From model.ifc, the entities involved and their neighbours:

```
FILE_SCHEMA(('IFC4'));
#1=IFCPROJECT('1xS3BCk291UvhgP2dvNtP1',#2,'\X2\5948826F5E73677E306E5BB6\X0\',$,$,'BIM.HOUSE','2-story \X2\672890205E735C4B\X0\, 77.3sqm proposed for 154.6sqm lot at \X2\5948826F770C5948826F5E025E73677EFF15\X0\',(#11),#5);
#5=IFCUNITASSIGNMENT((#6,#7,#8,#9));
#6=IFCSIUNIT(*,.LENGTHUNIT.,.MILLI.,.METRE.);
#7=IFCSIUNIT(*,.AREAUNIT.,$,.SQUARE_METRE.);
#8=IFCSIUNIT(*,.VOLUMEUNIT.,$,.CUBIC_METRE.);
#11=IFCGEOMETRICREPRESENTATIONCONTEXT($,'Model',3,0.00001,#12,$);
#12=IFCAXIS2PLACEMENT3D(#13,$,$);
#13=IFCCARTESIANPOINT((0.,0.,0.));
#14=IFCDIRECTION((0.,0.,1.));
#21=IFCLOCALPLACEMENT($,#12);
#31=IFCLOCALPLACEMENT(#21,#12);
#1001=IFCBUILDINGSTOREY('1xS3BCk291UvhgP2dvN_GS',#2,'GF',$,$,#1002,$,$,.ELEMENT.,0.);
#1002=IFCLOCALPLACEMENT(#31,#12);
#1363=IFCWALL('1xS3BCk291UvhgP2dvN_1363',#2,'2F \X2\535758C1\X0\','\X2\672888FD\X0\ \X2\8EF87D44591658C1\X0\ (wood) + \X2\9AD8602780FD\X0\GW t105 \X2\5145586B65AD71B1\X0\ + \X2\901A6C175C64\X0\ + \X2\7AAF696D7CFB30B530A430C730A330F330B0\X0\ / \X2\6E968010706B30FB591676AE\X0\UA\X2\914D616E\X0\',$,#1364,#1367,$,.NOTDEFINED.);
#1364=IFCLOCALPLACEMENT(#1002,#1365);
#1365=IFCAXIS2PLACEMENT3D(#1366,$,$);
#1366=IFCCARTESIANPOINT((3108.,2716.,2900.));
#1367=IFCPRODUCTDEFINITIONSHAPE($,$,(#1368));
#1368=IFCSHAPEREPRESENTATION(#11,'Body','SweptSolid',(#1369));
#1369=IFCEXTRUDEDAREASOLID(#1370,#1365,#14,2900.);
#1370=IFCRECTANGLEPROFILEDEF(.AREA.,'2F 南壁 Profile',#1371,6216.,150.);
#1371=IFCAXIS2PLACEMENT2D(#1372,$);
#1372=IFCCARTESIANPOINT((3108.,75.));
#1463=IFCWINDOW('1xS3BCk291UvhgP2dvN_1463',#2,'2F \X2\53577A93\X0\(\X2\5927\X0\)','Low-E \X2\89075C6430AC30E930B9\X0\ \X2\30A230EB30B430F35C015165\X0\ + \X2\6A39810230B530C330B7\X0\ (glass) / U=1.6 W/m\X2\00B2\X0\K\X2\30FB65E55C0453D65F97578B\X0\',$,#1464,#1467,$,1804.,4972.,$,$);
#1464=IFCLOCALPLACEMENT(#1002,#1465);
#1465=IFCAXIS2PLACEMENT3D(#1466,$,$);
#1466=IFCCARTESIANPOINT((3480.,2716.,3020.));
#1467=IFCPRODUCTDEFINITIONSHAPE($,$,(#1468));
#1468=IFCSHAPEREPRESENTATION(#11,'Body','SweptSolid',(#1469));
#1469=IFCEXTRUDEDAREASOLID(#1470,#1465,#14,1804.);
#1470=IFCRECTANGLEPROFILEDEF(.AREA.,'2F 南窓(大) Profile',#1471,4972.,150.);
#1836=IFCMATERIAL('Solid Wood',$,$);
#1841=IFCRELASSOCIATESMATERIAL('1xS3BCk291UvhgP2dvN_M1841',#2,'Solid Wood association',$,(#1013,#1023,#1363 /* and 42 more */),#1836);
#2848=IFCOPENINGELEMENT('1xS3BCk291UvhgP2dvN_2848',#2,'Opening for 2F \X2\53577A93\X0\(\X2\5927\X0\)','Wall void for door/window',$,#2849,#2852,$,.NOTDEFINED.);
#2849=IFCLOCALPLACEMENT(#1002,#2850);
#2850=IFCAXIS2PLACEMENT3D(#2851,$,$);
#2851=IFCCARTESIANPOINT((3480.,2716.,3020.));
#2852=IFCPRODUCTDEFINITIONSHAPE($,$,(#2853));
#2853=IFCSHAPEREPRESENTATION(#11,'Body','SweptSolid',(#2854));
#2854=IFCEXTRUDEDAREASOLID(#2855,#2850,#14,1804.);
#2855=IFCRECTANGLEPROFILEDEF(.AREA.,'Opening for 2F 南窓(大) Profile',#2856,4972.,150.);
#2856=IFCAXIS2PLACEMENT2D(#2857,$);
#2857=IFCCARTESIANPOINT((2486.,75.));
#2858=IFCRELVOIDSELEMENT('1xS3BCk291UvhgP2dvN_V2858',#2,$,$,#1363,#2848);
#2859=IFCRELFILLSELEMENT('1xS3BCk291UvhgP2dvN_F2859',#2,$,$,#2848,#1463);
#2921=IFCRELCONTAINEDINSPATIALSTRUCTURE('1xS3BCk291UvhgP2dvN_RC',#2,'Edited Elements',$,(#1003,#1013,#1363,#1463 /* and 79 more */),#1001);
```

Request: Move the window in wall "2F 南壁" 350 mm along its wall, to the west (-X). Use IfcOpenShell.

```python
import ifcopenshell
import ifcopenshell.api.geometry
import ifcopenshell.util.placement

model = ifcopenshell.open("model.ifc")

window = model.by_guid("1xS3BCk291UvhgP2dvN_1463")
opening = window.FillsVoids[0].RelatingOpeningElement
wall = opening.VoidsElements[0].RelatingBuildingElement

wall_matrix = ifcopenshell.util.placement.get_local_placement(wall.ObjectPlacement)
shift = wall_matrix[:3, 0] * -350.0
before = ifcopenshell.util.placement.get_local_placement(window.ObjectPlacement)[:3, 3].copy()

# The window is not placed relative to its opening, so move both.
for product in (opening, window):
    matrix = ifcopenshell.util.placement.get_local_placement(product.ObjectPlacement)
    matrix[:3, 3] += shift
    ifcopenshell.api.geometry.edit_object_placement(model, product=product, matrix=matrix, is_si=False)

after = ifcopenshell.util.placement.get_local_placement(window.ObjectPlacement)[:3, 3]
print("window moved by", (after - before).round(3) + 0.0)

model.write("model-out.ifc")
```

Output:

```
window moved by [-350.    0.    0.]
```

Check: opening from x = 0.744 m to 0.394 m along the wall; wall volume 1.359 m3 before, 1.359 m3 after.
